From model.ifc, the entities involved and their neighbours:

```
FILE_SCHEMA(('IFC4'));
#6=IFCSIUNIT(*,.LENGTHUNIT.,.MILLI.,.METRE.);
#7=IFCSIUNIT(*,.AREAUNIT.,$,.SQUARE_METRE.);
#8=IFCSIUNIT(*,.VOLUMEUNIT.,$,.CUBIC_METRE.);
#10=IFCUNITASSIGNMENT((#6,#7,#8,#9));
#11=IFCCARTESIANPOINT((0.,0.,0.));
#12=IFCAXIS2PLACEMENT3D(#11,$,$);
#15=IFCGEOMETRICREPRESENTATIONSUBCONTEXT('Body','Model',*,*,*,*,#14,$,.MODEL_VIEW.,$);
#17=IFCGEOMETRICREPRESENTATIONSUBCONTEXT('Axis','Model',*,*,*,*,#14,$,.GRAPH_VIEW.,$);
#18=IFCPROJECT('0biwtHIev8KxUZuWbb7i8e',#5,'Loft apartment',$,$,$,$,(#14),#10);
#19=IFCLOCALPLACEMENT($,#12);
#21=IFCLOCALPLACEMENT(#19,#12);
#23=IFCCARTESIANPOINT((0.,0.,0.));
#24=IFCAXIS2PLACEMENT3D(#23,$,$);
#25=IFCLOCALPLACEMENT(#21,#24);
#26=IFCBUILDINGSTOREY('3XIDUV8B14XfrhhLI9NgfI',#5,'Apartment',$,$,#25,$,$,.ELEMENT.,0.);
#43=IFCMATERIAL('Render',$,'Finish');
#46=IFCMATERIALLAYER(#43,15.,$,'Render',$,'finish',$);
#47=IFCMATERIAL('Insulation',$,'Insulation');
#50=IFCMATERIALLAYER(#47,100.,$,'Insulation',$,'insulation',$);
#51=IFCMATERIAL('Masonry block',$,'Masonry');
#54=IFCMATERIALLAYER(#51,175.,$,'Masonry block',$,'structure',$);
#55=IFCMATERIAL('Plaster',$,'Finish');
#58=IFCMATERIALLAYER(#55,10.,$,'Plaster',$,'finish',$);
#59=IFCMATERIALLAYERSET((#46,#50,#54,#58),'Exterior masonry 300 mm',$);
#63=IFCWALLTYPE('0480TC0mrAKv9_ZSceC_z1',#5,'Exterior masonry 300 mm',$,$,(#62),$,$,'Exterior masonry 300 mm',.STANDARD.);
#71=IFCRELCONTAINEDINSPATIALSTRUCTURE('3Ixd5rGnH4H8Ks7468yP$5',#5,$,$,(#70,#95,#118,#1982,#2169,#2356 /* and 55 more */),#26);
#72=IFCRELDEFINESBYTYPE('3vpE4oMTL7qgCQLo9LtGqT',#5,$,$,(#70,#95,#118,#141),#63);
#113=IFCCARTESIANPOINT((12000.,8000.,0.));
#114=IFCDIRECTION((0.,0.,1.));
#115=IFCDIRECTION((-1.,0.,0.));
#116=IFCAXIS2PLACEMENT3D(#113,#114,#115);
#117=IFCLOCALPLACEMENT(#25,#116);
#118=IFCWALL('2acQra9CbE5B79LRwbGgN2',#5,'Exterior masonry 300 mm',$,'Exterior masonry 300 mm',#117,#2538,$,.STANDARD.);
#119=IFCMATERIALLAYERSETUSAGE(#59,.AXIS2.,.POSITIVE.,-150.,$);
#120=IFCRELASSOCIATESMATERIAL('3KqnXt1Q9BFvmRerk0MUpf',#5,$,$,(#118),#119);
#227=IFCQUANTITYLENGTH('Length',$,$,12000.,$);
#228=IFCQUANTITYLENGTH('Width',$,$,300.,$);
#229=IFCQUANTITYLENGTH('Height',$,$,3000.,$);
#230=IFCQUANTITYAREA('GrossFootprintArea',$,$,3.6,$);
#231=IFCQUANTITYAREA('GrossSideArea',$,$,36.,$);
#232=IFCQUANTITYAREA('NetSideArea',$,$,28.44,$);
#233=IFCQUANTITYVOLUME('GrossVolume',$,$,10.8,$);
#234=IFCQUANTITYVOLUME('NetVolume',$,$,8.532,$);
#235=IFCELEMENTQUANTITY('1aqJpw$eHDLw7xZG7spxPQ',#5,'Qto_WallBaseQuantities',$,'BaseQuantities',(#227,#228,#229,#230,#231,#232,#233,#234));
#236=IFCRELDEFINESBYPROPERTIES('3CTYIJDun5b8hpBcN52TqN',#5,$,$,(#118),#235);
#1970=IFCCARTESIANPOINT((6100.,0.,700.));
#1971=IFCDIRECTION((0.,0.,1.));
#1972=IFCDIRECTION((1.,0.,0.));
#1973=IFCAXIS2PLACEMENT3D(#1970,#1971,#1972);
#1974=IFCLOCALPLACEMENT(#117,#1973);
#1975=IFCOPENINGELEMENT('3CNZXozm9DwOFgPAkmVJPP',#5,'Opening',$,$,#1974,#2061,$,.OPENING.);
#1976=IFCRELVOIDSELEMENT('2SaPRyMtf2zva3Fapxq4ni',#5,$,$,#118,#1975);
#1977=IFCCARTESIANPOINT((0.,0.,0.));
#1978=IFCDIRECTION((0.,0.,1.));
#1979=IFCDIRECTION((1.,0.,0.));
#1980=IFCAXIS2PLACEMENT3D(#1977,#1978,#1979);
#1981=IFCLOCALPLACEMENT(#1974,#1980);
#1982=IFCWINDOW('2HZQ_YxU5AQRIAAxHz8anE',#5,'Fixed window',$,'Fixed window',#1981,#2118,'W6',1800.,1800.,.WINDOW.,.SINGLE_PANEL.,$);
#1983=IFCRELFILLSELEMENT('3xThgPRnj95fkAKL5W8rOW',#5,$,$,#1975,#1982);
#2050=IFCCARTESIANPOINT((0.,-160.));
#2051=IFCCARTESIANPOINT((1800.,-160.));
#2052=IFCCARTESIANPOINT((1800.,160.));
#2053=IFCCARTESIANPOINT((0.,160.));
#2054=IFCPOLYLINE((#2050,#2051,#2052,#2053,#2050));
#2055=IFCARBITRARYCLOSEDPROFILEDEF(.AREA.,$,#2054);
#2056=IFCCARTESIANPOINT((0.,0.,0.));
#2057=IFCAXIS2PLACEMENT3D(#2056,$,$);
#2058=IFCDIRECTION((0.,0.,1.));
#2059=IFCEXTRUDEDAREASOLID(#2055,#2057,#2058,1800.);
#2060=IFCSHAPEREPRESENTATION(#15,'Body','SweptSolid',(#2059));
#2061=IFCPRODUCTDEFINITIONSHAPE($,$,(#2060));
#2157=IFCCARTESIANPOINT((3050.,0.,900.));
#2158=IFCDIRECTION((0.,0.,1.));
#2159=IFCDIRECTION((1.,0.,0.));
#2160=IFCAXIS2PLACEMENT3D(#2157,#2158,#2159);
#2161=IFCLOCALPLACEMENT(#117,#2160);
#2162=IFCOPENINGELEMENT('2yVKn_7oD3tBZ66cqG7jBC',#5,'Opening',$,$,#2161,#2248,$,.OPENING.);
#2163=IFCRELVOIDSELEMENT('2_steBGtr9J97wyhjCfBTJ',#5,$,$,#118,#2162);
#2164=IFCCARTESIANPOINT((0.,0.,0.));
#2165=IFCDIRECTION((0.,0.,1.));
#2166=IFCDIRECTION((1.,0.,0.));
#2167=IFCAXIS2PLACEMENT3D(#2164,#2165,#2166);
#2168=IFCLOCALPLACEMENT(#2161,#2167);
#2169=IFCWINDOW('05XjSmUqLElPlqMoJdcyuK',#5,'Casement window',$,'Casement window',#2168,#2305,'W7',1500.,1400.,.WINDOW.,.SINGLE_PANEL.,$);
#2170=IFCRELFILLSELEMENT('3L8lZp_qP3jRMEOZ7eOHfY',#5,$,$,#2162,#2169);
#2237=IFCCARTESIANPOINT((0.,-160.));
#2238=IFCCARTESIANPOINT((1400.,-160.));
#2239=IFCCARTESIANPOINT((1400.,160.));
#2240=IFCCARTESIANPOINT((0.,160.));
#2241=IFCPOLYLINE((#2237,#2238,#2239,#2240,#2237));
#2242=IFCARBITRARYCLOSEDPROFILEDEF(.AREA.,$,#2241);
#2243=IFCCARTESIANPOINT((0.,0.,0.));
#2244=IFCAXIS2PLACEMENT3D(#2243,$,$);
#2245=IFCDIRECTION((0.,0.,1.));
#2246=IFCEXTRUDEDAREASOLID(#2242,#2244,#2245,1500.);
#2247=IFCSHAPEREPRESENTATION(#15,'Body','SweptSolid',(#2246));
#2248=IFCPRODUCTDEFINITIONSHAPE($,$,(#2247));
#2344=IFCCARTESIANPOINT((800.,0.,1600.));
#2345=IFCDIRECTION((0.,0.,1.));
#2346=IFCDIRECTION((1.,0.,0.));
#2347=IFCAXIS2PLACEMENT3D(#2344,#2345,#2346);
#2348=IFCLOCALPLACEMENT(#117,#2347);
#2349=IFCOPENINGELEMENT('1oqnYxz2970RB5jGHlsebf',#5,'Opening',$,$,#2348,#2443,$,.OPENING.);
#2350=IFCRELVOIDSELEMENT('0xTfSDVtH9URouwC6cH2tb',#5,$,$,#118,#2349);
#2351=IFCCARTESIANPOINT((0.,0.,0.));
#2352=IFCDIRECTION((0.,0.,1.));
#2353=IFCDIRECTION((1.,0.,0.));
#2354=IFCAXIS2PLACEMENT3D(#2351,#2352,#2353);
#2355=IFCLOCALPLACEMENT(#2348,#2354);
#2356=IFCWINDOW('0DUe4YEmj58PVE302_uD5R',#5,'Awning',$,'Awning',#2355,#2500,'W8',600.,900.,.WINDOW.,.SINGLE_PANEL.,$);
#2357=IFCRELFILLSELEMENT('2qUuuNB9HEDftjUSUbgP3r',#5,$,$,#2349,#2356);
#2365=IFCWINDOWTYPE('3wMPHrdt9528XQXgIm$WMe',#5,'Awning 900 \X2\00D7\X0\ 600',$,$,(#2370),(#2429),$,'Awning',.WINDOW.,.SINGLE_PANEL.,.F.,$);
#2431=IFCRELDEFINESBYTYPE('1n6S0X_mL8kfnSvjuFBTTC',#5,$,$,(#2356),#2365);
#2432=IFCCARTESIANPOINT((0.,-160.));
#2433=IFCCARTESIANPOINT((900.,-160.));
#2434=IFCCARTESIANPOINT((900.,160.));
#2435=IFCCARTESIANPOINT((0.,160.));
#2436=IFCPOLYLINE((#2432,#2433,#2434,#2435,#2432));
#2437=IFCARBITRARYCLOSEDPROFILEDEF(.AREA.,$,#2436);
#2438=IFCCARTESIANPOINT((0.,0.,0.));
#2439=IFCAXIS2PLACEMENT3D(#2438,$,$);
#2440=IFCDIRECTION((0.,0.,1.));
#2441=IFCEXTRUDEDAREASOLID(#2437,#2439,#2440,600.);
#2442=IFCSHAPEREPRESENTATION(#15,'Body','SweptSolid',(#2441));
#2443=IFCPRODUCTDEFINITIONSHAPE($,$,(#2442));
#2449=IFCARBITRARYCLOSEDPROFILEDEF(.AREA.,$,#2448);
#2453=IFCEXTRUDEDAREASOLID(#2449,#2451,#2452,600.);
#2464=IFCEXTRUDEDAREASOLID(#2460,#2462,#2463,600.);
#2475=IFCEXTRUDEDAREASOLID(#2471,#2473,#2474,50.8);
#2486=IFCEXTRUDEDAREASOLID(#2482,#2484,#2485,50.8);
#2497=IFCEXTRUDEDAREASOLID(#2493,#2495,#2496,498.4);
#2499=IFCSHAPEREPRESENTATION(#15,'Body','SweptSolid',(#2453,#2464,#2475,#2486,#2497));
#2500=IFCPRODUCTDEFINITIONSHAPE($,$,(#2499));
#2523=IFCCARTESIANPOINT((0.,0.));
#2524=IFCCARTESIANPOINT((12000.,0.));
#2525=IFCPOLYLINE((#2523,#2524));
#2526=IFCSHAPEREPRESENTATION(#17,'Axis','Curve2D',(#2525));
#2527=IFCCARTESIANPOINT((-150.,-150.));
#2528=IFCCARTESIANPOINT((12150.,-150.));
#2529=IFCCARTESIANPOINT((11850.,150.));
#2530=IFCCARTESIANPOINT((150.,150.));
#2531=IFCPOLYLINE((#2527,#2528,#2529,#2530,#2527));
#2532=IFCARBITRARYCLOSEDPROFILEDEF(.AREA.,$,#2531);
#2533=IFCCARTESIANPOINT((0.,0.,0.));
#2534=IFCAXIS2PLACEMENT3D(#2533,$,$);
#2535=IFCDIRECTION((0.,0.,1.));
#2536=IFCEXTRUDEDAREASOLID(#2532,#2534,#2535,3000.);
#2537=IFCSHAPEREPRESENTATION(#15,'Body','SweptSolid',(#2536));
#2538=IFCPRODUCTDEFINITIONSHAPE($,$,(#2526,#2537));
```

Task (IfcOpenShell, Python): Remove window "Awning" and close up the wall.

```python
import ifcopenshell
import ifcopenshell.api.feature
import ifcopenshell.api.pset
import ifcopenshell.api.root
import ifcopenshell.geom
import ifcopenshell.util.element
import ifcopenshell.util.shape
import ifcopenshell.util.unit

model = ifcopenshell.open("model.ifc")
area_scale = ifcopenshell.util.unit.calculate_unit_scale(model, "AREAUNIT")
volume_scale = ifcopenshell.util.unit.calculate_unit_scale(model, "VOLUMEUNIT")
settings = ifcopenshell.geom.settings()


def volume(element):
    """Net volume in cubic metres, openings subtracted."""
    shape = ifcopenshell.geom.create_shape(settings, element)
    return ifcopenshell.util.shape.get_volume(shape.geometry)


window = model.by_guid("0DUe4YEmj58PVE302_uD5R")
opening = window.FillsVoids[0].RelatingOpeningElement
wall = opening.VoidsElements[0].RelatingBuildingElement
before = volume(wall)

ifcopenshell.api.root.remove_product(model, product=window)
ifcopenshell.api.feature.remove_feature(model, feature=opening)

after = volume(wall)
thickness = 0.3  # wall thickness in metres

# Update the wall's stored quantities.
qto = model.by_id(ifcopenshell.util.element.get_pset(wall, "Qto_WallBaseQuantities", should_inherit=False)["id"])
ifcopenshell.api.pset.edit_qto(model, qto=qto, properties={
    "NetSideArea": after / thickness / area_scale,
    "NetVolume": after / volume_scale,
})

print(f"wall volume {before:.3f} -> {after:.3f} m3")

model.write("model_edited.ifc")
```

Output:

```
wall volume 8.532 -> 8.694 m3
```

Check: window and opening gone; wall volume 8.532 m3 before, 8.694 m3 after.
